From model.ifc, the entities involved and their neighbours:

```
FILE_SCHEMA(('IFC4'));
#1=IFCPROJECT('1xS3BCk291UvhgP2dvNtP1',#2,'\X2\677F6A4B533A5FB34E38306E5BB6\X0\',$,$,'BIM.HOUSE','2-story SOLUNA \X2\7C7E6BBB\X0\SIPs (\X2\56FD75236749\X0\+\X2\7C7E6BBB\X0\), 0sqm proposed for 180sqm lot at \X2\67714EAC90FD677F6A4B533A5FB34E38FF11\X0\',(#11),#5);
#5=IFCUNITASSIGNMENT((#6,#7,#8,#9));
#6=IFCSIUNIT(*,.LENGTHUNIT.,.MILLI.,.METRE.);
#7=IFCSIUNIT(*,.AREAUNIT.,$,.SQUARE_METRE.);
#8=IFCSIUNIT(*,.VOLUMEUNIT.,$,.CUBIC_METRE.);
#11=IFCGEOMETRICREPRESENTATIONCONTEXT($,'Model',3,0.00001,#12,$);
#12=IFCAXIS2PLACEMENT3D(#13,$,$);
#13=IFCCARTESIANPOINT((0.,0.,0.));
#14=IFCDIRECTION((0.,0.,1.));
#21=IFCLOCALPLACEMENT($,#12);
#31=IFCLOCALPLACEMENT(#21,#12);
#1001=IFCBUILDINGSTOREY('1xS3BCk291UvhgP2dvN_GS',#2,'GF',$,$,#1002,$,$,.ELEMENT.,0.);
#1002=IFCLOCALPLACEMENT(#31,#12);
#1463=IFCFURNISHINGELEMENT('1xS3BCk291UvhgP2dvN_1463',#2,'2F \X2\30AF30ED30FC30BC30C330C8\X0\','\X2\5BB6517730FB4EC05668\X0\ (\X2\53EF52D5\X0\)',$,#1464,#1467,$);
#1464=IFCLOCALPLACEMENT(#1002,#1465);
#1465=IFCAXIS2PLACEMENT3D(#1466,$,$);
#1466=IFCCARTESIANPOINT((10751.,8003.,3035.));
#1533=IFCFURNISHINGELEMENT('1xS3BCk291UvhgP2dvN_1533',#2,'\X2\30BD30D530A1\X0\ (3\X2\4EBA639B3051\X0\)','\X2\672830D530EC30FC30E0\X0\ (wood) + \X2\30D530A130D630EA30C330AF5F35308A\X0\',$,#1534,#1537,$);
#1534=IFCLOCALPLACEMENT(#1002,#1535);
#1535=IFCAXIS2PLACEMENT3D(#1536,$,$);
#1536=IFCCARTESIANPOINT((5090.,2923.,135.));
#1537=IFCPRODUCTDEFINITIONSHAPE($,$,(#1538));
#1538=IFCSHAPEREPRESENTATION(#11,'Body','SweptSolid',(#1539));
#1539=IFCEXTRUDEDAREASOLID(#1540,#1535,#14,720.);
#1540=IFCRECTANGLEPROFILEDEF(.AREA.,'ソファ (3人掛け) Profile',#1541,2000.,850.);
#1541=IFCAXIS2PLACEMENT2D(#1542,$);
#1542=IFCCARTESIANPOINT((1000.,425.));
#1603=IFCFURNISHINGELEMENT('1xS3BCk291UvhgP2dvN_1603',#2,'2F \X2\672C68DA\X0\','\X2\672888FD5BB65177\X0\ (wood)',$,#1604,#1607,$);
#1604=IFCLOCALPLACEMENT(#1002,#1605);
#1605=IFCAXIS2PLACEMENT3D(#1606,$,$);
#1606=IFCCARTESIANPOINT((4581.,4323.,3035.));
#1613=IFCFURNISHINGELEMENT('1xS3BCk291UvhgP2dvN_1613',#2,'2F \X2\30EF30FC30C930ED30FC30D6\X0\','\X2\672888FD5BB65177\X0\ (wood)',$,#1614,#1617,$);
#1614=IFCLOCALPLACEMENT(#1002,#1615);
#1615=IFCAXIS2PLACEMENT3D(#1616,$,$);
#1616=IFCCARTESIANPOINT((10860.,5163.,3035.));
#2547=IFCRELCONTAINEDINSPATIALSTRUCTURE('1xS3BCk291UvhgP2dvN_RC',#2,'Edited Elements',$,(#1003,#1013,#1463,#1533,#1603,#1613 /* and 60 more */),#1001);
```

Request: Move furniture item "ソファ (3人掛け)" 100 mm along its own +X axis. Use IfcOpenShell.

```python
import ifcopenshell
import ifcopenshell.api.geometry
import ifcopenshell.util.placement
import ifcopenshell.util.unit

model = ifcopenshell.open("model.ifc")
unit_scale = ifcopenshell.util.unit.calculate_unit_scale(model)

item = model.by_id(1533)
matrix = ifcopenshell.util.placement.get_local_placement(item.ObjectPlacement)
matrix[:3, 3] += matrix[:3, 0] * 0.1 / unit_scale
ifcopenshell.api.geometry.edit_object_placement(model, product=item, matrix=matrix, is_si=False)

print(ifcopenshell.util.placement.get_local_placement(item.ObjectPlacement).round(3) + 0.0)

model.write("model-out.ifc")
```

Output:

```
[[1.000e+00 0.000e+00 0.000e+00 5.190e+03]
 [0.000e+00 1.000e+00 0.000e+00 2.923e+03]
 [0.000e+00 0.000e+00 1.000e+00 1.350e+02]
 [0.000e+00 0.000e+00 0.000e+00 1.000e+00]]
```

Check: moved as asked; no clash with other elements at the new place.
